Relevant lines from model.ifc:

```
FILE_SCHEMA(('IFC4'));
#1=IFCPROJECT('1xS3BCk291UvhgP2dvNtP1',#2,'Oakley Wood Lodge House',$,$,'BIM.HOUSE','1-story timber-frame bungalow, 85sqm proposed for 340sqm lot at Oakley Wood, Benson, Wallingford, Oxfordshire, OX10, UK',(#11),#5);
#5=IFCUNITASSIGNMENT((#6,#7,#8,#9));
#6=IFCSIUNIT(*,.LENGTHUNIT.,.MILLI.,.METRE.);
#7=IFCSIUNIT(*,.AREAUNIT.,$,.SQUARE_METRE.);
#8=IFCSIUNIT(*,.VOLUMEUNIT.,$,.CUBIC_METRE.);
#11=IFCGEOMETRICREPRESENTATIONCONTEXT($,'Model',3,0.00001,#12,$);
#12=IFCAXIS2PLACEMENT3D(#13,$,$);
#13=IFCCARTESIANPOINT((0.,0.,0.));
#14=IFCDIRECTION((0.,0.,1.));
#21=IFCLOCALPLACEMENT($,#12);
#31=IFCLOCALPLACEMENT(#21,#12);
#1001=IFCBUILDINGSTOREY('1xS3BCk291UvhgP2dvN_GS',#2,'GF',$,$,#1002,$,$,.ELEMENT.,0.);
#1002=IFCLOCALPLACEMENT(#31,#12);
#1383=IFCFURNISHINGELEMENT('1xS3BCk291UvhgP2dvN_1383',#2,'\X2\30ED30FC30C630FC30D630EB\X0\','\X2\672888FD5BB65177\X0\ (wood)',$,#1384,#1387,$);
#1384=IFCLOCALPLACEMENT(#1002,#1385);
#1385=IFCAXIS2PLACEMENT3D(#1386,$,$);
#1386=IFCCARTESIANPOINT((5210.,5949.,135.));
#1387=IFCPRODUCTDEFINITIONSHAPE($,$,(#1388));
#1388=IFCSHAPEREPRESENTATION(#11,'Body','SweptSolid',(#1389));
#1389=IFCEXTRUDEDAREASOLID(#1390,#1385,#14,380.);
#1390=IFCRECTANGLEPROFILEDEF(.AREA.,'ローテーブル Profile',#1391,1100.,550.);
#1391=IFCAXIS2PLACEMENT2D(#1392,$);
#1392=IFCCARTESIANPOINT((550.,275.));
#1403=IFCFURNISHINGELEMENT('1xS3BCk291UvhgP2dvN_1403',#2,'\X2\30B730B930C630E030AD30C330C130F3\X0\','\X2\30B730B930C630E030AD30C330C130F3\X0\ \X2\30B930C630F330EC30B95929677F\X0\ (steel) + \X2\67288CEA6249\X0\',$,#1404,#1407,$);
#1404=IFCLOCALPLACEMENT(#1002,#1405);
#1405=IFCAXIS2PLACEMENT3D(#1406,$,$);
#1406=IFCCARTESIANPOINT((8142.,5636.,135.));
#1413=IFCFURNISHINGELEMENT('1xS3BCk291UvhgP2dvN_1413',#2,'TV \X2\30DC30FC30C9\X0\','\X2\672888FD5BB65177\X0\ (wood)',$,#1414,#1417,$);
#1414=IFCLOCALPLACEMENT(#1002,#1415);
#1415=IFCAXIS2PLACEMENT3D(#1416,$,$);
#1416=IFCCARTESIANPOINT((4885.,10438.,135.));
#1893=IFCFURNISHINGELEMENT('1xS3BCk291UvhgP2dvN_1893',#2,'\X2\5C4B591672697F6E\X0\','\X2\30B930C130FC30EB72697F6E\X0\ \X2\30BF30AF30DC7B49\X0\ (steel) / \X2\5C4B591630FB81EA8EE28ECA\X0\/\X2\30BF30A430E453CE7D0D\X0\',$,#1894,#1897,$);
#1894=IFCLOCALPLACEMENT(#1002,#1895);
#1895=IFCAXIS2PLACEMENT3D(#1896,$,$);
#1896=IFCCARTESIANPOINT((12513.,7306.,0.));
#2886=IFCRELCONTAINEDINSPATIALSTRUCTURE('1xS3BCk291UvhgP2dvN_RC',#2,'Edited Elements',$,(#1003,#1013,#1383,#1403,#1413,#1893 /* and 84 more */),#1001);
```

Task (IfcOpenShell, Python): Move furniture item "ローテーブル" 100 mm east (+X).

```python
import ifcopenshell
import ifcopenshell.api.geometry
import ifcopenshell.util.placement
import ifcopenshell.util.unit

model = ifcopenshell.open("model.ifc")
unit_scale = ifcopenshell.util.unit.calculate_unit_scale(model)

item = model.by_guid("1xS3BCk291UvhgP2dvN_1383")
matrix = ifcopenshell.util.placement.get_local_placement(item.ObjectPlacement)
matrix[0, 3] += 0.1 / unit_scale
ifcopenshell.api.geometry.edit_object_placement(model, product=item, matrix=matrix, is_si=False)

print(ifcopenshell.util.placement.get_local_placement(item.ObjectPlacement).round(3) + 0.0)

model.write("model-out.ifc")
```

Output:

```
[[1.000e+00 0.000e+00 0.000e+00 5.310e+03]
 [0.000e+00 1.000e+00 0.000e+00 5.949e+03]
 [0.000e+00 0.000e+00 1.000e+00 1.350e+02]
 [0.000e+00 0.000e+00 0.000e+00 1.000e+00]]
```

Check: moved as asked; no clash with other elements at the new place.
